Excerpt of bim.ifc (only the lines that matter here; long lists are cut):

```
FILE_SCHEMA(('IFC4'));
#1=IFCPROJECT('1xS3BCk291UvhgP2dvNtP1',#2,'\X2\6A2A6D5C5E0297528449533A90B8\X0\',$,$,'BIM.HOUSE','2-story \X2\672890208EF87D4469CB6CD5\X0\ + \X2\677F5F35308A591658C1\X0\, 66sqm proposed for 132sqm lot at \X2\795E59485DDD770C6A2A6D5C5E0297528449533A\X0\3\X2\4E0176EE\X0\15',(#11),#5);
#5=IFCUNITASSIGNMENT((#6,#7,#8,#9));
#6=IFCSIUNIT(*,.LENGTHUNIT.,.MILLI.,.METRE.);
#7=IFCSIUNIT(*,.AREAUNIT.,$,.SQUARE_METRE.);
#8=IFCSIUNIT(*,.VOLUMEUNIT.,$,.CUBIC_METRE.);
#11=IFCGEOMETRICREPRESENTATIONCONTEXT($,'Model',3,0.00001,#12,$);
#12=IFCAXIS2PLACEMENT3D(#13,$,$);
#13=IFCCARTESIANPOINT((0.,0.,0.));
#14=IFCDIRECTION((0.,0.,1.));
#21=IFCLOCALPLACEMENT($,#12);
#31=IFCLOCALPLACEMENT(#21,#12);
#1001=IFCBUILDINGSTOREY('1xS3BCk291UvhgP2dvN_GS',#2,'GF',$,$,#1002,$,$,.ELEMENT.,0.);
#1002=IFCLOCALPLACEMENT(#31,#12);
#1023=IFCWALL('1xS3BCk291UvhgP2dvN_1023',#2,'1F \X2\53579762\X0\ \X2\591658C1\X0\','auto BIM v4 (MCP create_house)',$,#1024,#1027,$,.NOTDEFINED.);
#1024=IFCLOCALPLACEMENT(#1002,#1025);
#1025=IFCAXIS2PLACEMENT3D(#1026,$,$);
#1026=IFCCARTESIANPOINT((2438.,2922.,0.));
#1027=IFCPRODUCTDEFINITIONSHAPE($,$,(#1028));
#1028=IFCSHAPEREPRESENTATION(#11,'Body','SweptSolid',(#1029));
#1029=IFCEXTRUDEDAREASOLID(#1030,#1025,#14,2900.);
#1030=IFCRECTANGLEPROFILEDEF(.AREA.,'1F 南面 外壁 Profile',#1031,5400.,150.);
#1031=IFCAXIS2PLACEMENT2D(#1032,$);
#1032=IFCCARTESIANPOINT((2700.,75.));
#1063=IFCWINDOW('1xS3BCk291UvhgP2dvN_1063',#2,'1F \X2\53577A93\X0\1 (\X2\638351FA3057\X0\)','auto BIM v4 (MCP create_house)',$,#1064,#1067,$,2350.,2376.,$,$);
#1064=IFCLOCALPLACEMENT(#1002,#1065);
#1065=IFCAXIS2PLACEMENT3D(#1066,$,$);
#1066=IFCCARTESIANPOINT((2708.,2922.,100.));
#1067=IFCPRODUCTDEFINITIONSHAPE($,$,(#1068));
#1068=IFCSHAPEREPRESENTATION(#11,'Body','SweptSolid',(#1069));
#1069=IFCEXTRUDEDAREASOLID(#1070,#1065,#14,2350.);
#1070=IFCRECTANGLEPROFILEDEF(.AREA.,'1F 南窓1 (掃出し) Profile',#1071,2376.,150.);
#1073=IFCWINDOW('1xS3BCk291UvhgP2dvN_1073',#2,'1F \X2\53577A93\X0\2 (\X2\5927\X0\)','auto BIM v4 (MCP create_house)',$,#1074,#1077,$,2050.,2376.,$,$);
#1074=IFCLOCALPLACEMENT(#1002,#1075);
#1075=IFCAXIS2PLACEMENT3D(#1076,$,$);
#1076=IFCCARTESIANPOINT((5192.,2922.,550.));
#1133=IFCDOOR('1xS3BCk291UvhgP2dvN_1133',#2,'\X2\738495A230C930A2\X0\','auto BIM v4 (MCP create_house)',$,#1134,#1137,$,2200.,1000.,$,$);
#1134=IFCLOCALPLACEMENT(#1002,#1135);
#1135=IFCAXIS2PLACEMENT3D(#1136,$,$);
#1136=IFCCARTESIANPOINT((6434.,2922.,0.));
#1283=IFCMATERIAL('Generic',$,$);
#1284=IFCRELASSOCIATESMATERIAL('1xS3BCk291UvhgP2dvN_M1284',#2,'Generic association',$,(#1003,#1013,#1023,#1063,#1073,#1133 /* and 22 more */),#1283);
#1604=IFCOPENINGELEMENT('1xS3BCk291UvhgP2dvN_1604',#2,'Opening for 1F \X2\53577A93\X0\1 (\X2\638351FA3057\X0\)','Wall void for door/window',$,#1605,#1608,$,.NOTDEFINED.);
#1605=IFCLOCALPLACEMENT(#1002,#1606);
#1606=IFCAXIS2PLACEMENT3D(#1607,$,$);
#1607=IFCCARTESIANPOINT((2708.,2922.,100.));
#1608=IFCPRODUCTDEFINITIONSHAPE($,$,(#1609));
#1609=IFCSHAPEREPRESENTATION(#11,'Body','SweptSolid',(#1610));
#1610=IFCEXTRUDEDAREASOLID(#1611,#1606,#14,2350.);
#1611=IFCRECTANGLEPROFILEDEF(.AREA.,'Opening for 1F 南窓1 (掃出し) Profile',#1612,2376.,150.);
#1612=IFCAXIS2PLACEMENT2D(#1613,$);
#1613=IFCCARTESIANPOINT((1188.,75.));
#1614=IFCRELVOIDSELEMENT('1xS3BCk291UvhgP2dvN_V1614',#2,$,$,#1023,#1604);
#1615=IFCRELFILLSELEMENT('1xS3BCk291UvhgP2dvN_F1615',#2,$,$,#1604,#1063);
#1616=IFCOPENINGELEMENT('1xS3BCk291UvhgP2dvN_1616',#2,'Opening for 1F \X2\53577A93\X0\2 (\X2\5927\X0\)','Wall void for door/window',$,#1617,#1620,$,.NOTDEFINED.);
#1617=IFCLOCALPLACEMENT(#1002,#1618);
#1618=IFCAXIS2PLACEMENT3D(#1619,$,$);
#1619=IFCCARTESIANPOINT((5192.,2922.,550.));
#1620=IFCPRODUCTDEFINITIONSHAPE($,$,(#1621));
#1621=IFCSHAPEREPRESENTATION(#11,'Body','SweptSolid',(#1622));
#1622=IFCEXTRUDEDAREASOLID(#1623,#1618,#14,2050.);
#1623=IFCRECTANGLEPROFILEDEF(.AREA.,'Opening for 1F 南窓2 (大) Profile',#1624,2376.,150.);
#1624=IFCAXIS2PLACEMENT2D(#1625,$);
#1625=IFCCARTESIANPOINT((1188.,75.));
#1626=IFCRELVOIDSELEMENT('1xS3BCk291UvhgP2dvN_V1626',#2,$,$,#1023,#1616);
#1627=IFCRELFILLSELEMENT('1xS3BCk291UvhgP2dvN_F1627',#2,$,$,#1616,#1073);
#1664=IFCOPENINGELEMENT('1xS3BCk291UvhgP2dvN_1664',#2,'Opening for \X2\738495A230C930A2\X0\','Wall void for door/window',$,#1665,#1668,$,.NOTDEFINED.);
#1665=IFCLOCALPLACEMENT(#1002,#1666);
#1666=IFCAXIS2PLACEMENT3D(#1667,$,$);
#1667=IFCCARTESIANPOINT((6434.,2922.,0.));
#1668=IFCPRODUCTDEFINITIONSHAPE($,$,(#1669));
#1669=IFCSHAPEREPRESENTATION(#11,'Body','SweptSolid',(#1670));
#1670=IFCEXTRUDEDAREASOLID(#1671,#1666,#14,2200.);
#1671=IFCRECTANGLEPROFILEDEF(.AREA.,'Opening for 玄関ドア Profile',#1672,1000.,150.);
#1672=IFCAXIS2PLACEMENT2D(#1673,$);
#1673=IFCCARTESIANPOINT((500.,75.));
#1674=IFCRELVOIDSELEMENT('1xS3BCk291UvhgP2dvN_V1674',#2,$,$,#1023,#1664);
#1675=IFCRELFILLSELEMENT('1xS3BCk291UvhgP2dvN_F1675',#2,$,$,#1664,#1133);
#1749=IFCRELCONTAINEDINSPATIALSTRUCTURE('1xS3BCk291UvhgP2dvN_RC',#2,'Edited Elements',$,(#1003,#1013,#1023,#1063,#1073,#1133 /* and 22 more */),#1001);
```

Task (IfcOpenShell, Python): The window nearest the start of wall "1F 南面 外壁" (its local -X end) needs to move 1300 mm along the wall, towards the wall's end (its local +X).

```python
import ifcopenshell
import ifcopenshell.api.geometry
import ifcopenshell.util.placement

model = ifcopenshell.open("bim.ifc")

window = model.by_id(1063)
opening = window.FillsVoids[0].RelatingOpeningElement
wall = opening.VoidsElements[0].RelatingBuildingElement

wall_matrix = ifcopenshell.util.placement.get_local_placement(wall.ObjectPlacement)
shift = wall_matrix[:3, 0] * 1300.0
before = ifcopenshell.util.placement.get_local_placement(window.ObjectPlacement)[:3, 3].copy()

# The window is not placed relative to its opening, so move both.
for product in (opening, window):
    matrix = ifcopenshell.util.placement.get_local_placement(product.ObjectPlacement)
    matrix[:3, 3] += shift
    ifcopenshell.api.geometry.edit_object_placement(model, product=product, matrix=matrix, is_si=False)

after = ifcopenshell.util.placement.get_local_placement(window.ObjectPlacement)[:3, 3]
print("window moved by", (after - before).round(3) + 0.0)

model.write("bim_rev.ifc")
```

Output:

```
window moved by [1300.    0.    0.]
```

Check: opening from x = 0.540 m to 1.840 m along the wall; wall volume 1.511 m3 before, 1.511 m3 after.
